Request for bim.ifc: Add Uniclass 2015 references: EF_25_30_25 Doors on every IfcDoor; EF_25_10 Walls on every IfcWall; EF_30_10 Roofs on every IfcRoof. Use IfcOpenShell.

First a look at what the model holds.

```python
import ifcopenshell

model = ifcopenshell.open("bim.ifc")
print(model.schema)
print("classifications:", [c.Name for c in model.by_type("IfcClassification")])
for ifc_class in ("IfcDoor", "IfcRoof", "IfcStair", "IfcWall", "IfcWindow"):
    print(ifc_class, len(model.by_type(ifc_class)))
```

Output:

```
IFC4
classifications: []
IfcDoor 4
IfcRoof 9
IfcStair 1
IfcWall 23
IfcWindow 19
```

```python
import ifcopenshell
import ifcopenshell.api.classification

model = ifcopenshell.open("bim.ifc")

system = ifcopenshell.api.classification.add_classification(model, classification="Uniclass 2015")

codes = {
    "IfcDoor": ("EF_25_30_25", "Doors"),
    "IfcWall": ("EF_25_10", "Walls"),
    "IfcRoof": ("EF_30_10", "Roofs"),
}
for ifc_class, (code, name) in codes.items():
    products = model.by_type(ifc_class)
    ifcopenshell.api.classification.add_reference(
        model, products=products, classification=system, identification=code, name=name
    )
    print(code, len(products))

model.write("bim_updated.ifc")
```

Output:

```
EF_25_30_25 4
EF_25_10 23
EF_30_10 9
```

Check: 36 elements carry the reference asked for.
